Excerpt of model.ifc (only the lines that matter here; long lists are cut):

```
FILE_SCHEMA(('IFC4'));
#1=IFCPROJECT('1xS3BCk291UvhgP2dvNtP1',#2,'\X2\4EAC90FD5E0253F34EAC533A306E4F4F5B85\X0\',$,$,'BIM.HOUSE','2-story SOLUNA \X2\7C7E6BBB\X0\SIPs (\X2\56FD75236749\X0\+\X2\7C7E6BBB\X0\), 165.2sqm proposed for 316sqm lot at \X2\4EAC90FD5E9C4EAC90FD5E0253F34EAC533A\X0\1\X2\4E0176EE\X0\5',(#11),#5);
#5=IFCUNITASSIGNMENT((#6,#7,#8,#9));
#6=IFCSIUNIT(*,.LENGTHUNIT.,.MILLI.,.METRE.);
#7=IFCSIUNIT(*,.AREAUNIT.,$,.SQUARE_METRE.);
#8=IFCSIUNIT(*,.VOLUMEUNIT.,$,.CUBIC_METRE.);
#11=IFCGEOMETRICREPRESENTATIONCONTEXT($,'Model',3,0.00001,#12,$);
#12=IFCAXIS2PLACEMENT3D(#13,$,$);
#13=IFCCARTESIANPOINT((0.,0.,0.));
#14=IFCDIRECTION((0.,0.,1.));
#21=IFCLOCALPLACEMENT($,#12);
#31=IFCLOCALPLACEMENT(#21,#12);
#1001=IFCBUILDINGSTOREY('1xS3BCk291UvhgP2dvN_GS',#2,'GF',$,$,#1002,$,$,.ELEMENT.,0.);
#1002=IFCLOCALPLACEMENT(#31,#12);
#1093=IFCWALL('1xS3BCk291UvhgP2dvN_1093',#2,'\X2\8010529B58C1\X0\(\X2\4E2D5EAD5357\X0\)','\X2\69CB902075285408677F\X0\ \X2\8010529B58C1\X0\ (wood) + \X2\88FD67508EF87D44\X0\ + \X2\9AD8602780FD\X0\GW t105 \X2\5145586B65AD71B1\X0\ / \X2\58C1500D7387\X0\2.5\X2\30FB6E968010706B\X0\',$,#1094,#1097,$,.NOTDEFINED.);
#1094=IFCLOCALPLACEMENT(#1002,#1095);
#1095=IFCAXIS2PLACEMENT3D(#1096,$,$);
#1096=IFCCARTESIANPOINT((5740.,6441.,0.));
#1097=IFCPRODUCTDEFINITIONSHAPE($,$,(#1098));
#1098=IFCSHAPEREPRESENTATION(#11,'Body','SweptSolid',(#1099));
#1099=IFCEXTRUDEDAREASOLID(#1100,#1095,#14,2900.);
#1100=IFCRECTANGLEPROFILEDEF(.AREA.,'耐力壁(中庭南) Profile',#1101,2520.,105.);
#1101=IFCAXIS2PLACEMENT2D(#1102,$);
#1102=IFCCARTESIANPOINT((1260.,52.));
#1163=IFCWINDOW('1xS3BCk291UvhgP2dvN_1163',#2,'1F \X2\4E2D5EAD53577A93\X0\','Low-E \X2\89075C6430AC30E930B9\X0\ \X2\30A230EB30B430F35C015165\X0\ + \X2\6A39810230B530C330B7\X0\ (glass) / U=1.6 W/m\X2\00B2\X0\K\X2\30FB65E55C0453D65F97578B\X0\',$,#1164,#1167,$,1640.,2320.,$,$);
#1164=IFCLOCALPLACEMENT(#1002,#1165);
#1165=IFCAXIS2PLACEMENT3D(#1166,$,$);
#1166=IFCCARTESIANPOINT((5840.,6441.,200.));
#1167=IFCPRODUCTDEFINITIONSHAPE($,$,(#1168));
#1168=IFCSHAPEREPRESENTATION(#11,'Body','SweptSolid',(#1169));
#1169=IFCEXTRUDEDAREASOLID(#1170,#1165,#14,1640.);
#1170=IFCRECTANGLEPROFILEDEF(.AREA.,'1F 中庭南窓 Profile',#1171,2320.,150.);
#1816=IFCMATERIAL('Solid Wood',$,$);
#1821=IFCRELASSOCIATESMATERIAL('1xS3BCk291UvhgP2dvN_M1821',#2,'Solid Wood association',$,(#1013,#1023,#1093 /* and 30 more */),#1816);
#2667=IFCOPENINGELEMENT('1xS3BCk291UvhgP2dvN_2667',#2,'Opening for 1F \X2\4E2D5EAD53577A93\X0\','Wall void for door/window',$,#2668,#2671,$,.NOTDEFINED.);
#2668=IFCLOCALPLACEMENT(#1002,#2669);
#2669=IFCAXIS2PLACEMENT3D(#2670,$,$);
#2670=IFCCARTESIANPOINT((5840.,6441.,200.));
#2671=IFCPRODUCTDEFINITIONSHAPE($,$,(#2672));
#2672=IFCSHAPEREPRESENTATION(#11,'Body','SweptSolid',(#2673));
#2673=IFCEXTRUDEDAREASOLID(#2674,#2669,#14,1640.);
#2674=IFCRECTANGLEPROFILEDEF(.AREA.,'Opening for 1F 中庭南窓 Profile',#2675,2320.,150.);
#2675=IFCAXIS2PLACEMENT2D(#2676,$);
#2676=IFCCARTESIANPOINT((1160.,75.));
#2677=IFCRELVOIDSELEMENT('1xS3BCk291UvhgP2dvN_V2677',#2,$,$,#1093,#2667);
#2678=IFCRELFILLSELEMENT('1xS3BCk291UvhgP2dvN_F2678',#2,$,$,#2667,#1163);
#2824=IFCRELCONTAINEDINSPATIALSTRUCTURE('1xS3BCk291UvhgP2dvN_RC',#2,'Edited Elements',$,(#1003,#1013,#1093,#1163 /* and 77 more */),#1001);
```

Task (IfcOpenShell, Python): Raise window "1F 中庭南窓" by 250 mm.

```python
import numpy as np
import ifcopenshell
import ifcopenshell.api.geometry
import ifcopenshell.util.placement
import ifcopenshell.util.unit

model = ifcopenshell.open("model.ifc")
unit_scale = ifcopenshell.util.unit.calculate_unit_scale(model)

window = model.by_guid("1xS3BCk291UvhgP2dvN_1163")
opening = window.FillsVoids[0].RelatingOpeningElement
dz = 0.25 / unit_scale

shift = np.array([0.0, 0.0, dz])
# The window is not placed relative to its opening, so move both.
for product in (opening, window):
    matrix = ifcopenshell.util.placement.get_local_placement(product.ObjectPlacement)
    matrix[:3, 3] += shift
    ifcopenshell.api.geometry.edit_object_placement(model, product=product, matrix=matrix, is_si=False)

print(f"moved by {dz * unit_scale:+.3f} m")

model.write("model_v2.ifc")
```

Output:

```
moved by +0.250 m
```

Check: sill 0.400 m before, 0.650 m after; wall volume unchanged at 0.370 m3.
